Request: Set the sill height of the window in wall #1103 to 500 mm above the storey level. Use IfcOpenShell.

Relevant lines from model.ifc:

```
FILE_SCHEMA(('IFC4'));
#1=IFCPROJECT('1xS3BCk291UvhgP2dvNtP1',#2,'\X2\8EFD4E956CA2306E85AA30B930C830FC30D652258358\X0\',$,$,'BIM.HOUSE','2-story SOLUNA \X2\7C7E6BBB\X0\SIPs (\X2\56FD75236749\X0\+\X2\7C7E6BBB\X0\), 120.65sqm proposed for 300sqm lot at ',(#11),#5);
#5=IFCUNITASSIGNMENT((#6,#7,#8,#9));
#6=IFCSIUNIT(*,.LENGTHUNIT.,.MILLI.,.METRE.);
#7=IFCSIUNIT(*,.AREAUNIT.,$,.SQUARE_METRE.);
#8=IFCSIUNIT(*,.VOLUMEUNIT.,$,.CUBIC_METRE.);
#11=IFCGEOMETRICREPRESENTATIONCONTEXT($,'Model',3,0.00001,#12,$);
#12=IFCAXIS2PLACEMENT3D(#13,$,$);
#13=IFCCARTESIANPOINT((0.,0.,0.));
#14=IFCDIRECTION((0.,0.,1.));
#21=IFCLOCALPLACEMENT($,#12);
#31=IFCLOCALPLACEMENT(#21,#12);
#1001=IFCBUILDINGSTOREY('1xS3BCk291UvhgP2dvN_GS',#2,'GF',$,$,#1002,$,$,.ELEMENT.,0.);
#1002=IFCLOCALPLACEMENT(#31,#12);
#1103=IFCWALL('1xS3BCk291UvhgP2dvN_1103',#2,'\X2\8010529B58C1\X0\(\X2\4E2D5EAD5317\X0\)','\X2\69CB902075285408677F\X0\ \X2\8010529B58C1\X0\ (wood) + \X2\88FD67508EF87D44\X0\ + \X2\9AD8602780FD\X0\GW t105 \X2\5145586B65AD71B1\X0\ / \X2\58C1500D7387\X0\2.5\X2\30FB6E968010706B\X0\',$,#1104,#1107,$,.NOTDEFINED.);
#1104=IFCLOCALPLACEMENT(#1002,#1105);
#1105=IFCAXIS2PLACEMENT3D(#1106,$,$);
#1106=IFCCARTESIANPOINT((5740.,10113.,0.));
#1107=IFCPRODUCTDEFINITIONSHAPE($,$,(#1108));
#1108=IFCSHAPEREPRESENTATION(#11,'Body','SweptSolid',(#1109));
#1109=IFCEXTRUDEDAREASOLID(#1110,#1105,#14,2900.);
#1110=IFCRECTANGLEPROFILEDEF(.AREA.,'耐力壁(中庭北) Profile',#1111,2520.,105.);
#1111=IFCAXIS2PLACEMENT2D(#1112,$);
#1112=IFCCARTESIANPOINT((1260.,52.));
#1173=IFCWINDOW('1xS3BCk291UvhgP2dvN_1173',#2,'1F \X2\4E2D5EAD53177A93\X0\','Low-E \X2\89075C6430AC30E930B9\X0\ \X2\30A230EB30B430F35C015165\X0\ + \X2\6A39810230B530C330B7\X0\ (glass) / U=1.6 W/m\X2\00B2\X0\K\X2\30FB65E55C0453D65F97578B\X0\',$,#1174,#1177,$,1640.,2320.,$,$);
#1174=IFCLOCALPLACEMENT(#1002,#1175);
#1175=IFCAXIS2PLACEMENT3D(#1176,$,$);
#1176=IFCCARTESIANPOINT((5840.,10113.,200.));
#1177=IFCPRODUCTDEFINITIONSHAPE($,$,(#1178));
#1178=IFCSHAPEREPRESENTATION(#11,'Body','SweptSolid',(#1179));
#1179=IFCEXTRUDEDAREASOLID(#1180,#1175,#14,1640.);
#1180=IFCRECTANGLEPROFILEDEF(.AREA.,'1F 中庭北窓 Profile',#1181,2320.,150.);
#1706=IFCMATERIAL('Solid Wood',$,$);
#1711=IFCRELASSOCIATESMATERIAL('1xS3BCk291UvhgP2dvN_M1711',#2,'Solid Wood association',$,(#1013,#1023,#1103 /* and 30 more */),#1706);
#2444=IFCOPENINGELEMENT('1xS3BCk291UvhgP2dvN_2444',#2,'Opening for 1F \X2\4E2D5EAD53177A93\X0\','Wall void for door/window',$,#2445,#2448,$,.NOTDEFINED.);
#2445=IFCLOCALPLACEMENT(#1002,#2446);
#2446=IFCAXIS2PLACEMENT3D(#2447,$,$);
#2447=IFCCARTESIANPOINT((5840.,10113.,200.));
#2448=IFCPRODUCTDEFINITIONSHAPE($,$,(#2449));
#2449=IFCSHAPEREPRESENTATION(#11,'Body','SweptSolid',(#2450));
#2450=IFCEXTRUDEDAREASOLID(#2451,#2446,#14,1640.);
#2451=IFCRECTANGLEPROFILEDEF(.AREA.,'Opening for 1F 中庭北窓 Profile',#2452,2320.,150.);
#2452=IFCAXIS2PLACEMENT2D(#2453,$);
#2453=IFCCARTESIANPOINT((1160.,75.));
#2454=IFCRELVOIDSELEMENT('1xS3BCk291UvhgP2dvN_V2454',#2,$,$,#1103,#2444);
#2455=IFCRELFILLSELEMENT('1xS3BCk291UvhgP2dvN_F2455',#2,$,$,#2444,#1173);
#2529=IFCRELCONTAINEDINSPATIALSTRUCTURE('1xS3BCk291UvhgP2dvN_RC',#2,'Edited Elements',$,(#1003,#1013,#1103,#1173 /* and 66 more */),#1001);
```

```python
import numpy as np
import ifcopenshell
import ifcopenshell.api.geometry
import ifcopenshell.geom
import ifcopenshell.util.element
import ifcopenshell.util.placement
import ifcopenshell.util.shape
import ifcopenshell.util.unit

model = ifcopenshell.open("model.ifc")
unit_scale = ifcopenshell.util.unit.calculate_unit_scale(model)

window = model.by_guid("1xS3BCk291UvhgP2dvN_1173")
opening = window.FillsVoids[0].RelatingOpeningElement
storey = ifcopenshell.util.element.get_container(window, ifc_class="IfcBuildingStorey")
level = ifcopenshell.util.placement.get_local_placement(storey.ObjectPlacement)[2, 3]

# The opening's origin need not be at the sill, so measure its lowest point.
shape = ifcopenshell.geom.create_shape(ifcopenshell.geom.settings(), opening)
bottom = ifcopenshell.util.shape.get_shape_bottom_elevation(shape, shape.geometry) / unit_scale
dz = level + 0.5 / unit_scale - bottom

shift = np.array([0.0, 0.0, dz])
# The window is not placed relative to its opening, so move both.
for product in (opening, window):
    matrix = ifcopenshell.util.placement.get_local_placement(product.ObjectPlacement)
    matrix[:3, 3] += shift
    ifcopenshell.api.geometry.edit_object_placement(model, product=product, matrix=matrix, is_si=False)

print(f"moved by {dz * unit_scale:+.3f} m")

model.write("model_v2.ifc")
```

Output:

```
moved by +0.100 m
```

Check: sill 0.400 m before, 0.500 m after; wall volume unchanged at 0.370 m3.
